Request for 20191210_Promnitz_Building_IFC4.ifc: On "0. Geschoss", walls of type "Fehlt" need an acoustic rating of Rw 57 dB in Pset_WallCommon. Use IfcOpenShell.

First a look at what the model holds.

```python
import ifcopenshell
import ifcopenshell.util.element

model = ifcopenshell.open("20191210_Promnitz_Building_IFC4.ifc")
print(model.schema)
storey = next(s for s in model.by_type("IfcBuildingStorey") if s.Name == "0. Geschoss")
walls = [e for e in ifcopenshell.util.element.get_decomposition(storey) if e.is_a("IfcWall")]
seen = {}
for e in walls:
    element_type = ifcopenshell.util.element.get_type(e)
    key = (element_type.Name if element_type != e and element_type else None, ifcopenshell.util.element.get_pset(e, "Pset_WallCommon", "AcousticRating"))
    seen[key] = seen.get(key, 0) + 1
for (name, value), count in sorted(seen.items(), key=str):
    print(count, "x", name, "|", value)
```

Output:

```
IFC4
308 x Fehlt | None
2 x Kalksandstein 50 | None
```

```python
import ifcopenshell
import ifcopenshell.api.pset
import ifcopenshell.util.element

model = ifcopenshell.open("20191210_Promnitz_Building_IFC4.ifc")

storey = next(s for s in model.by_type("IfcBuildingStorey") if s.Name == "0. Geschoss")
walls = [e for e in ifcopenshell.util.element.get_decomposition(storey) if e.is_a("IfcWall")]

count = 0
for e in walls:
    element_type = ifcopenshell.util.element.get_type(e)
    if element_type in (None, e) or element_type.Name != "Fehlt":
        continue
    # add_pset returns the element's existing set when there is one.
    pset = ifcopenshell.api.pset.add_pset(model, product=e, name="Pset_WallCommon")
    ifcopenshell.api.pset.edit_pset(model, pset=pset, properties={"AcousticRating": "Rw 57 dB"})
    count += 1

print(count, "walls updated")

model.write("20191210_Promnitz_Building_IFC4_v2.ifc")
```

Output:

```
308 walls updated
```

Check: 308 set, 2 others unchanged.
